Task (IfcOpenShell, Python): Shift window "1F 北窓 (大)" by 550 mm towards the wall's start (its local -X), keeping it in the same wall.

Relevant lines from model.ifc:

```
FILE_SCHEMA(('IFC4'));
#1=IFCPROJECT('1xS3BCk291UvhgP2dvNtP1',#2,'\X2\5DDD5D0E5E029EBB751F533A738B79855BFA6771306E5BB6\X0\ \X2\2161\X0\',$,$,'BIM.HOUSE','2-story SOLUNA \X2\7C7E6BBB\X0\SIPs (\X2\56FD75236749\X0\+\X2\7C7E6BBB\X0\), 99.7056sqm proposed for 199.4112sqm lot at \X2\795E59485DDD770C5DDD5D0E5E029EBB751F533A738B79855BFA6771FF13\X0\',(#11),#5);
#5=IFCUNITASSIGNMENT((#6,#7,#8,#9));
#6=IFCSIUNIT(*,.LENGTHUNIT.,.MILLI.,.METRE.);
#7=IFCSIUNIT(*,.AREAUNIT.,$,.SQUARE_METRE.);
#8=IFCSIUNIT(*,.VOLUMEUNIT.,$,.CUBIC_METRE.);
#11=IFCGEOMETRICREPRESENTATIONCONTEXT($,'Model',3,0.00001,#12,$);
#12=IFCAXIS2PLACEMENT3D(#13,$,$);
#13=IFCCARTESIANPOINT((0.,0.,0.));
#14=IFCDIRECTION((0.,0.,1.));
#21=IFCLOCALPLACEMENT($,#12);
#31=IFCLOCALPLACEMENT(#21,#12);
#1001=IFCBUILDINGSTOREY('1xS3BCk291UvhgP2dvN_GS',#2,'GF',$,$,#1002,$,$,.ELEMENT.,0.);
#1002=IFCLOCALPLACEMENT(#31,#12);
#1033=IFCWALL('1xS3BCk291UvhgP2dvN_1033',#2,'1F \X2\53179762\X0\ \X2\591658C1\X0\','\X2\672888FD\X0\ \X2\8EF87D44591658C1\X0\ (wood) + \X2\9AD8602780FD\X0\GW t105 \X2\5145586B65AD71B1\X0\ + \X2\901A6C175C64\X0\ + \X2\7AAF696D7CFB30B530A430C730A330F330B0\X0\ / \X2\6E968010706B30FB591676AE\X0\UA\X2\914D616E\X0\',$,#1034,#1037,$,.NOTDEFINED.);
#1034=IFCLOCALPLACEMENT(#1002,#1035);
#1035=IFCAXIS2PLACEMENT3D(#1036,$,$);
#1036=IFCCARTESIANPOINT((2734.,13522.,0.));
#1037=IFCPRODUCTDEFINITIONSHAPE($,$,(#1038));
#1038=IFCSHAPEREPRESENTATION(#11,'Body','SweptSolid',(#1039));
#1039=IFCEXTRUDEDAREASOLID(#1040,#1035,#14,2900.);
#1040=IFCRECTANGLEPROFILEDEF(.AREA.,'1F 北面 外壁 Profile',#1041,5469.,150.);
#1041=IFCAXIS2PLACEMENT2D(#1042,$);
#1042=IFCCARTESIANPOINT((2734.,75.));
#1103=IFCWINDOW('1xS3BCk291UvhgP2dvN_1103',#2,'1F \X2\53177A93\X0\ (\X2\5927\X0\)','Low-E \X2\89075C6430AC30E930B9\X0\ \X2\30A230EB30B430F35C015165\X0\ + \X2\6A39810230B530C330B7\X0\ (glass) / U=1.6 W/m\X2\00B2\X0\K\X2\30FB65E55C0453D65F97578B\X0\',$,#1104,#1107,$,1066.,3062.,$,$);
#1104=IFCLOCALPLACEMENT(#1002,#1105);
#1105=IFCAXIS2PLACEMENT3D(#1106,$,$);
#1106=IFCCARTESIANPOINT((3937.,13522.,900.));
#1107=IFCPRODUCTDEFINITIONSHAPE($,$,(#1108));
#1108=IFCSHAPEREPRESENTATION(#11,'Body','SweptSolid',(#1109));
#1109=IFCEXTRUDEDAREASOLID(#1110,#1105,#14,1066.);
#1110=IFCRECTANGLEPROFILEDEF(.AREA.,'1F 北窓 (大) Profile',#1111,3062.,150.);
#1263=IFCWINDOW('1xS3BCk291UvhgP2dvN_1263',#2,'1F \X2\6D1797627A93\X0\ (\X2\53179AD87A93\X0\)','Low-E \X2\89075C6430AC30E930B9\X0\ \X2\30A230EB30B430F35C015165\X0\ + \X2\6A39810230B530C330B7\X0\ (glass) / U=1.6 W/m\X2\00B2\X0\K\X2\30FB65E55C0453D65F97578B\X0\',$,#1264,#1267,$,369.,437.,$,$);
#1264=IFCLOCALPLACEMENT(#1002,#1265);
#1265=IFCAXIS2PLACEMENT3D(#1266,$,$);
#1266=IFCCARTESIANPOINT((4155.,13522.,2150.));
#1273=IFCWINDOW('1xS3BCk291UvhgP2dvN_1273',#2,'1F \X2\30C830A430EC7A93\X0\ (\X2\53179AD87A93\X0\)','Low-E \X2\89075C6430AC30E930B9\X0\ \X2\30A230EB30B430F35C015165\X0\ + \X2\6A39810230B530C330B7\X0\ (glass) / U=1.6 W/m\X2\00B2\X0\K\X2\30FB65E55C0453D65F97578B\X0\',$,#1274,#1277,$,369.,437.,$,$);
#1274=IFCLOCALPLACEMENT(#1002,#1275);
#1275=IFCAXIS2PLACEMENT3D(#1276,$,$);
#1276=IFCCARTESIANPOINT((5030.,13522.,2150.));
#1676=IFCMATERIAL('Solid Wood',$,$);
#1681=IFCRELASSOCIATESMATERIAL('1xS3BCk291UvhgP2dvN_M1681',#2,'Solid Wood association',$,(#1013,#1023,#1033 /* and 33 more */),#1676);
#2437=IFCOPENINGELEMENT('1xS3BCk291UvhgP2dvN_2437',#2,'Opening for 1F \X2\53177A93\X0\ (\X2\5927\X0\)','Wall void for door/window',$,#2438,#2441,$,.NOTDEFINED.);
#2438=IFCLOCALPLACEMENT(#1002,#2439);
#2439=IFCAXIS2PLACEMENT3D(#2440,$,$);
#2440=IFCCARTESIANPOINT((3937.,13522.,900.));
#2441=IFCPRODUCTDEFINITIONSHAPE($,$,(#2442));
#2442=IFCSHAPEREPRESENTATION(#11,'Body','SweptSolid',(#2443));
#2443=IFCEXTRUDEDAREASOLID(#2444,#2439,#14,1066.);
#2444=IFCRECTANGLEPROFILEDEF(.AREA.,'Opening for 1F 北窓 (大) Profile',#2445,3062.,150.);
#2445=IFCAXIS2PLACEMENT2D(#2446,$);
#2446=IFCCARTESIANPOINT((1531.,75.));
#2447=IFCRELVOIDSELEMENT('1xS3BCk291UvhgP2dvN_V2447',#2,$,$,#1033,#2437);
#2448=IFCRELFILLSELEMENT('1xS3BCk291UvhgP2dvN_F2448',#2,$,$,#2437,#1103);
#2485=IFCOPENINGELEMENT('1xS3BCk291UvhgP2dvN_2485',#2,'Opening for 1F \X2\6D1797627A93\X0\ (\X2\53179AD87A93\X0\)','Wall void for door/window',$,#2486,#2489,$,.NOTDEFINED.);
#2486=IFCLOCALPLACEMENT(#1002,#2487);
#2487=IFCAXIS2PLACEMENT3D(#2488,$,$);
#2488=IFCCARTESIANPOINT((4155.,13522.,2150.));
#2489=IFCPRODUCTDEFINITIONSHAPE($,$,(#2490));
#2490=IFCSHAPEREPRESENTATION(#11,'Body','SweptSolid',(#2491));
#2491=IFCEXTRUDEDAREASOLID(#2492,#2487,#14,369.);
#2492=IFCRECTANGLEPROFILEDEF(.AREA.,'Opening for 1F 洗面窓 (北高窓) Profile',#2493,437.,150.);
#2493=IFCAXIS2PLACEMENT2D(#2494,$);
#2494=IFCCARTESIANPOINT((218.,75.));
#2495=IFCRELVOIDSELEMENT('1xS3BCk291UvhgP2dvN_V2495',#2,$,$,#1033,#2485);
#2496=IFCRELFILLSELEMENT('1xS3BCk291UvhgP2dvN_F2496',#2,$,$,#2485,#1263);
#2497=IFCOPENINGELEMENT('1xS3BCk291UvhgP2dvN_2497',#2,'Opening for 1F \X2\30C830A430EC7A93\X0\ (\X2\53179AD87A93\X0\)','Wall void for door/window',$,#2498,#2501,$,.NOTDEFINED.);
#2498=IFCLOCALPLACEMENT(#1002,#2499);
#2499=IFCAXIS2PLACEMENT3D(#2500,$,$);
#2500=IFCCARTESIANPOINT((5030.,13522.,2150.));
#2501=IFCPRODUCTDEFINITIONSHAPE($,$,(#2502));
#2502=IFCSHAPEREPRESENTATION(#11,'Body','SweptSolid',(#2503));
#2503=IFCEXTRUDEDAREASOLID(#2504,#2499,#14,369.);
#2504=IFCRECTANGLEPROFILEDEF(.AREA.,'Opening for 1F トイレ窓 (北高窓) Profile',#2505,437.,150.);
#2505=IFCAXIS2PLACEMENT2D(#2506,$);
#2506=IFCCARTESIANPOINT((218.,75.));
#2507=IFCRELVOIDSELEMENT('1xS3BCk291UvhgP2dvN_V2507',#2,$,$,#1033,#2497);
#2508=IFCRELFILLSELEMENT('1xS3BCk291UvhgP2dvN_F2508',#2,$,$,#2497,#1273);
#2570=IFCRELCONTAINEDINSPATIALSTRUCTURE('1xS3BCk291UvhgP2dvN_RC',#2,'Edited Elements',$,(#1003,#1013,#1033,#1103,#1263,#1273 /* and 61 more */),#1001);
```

```python
import ifcopenshell
import ifcopenshell.api.geometry
import ifcopenshell.util.placement

model = ifcopenshell.open("model.ifc")

window = model.by_guid("1xS3BCk291UvhgP2dvN_1103")
opening = window.FillsVoids[0].RelatingOpeningElement
wall = opening.VoidsElements[0].RelatingBuildingElement

wall_matrix = ifcopenshell.util.placement.get_local_placement(wall.ObjectPlacement)
shift = wall_matrix[:3, 0] * -550.0
before = ifcopenshell.util.placement.get_local_placement(window.ObjectPlacement)[:3, 3].copy()

# The window is not placed relative to its opening, so move both.
for product in (opening, window):
    matrix = ifcopenshell.util.placement.get_local_placement(product.ObjectPlacement)
    matrix[:3, 3] += shift
    ifcopenshell.api.geometry.edit_object_placement(model, product=product, matrix=matrix, is_si=False)

after = ifcopenshell.util.placement.get_local_placement(window.ObjectPlacement)[:3, 3]
print("window moved by", (after - before).round(3) + 0.0)

model.write("model_v2.ifc")
```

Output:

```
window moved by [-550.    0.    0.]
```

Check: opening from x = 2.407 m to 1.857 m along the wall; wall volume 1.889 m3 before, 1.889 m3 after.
